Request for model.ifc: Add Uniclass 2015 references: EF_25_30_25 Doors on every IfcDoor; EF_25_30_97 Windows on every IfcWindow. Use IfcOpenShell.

First a look at what the model holds.

```python
import ifcopenshell

model = ifcopenshell.open("model.ifc")
print(model.schema)
print("classifications:", [c.Name for c in model.by_type("IfcClassification")])
for ifc_class in ("IfcDoor", "IfcRoof", "IfcStair", "IfcWall", "IfcWindow"):
    print(ifc_class, len(model.by_type(ifc_class)))
```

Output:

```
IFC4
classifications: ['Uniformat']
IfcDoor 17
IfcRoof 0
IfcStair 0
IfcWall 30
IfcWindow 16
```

```python
import ifcopenshell
import ifcopenshell.api.classification

model = ifcopenshell.open("model.ifc")

system = ifcopenshell.api.classification.add_classification(model, classification="Uniclass 2015")

codes = {
    "IfcDoor": ("EF_25_30_25", "Doors"),
    "IfcWindow": ("EF_25_30_97", "Windows"),
}
for ifc_class, (code, name) in codes.items():
    products = model.by_type(ifc_class)
    ifcopenshell.api.classification.add_reference(
        model, products=products, classification=system, identification=code, name=name
    )
    print(code, len(products))

model.write("model-out.ifc")
```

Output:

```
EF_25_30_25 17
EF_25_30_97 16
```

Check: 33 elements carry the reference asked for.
